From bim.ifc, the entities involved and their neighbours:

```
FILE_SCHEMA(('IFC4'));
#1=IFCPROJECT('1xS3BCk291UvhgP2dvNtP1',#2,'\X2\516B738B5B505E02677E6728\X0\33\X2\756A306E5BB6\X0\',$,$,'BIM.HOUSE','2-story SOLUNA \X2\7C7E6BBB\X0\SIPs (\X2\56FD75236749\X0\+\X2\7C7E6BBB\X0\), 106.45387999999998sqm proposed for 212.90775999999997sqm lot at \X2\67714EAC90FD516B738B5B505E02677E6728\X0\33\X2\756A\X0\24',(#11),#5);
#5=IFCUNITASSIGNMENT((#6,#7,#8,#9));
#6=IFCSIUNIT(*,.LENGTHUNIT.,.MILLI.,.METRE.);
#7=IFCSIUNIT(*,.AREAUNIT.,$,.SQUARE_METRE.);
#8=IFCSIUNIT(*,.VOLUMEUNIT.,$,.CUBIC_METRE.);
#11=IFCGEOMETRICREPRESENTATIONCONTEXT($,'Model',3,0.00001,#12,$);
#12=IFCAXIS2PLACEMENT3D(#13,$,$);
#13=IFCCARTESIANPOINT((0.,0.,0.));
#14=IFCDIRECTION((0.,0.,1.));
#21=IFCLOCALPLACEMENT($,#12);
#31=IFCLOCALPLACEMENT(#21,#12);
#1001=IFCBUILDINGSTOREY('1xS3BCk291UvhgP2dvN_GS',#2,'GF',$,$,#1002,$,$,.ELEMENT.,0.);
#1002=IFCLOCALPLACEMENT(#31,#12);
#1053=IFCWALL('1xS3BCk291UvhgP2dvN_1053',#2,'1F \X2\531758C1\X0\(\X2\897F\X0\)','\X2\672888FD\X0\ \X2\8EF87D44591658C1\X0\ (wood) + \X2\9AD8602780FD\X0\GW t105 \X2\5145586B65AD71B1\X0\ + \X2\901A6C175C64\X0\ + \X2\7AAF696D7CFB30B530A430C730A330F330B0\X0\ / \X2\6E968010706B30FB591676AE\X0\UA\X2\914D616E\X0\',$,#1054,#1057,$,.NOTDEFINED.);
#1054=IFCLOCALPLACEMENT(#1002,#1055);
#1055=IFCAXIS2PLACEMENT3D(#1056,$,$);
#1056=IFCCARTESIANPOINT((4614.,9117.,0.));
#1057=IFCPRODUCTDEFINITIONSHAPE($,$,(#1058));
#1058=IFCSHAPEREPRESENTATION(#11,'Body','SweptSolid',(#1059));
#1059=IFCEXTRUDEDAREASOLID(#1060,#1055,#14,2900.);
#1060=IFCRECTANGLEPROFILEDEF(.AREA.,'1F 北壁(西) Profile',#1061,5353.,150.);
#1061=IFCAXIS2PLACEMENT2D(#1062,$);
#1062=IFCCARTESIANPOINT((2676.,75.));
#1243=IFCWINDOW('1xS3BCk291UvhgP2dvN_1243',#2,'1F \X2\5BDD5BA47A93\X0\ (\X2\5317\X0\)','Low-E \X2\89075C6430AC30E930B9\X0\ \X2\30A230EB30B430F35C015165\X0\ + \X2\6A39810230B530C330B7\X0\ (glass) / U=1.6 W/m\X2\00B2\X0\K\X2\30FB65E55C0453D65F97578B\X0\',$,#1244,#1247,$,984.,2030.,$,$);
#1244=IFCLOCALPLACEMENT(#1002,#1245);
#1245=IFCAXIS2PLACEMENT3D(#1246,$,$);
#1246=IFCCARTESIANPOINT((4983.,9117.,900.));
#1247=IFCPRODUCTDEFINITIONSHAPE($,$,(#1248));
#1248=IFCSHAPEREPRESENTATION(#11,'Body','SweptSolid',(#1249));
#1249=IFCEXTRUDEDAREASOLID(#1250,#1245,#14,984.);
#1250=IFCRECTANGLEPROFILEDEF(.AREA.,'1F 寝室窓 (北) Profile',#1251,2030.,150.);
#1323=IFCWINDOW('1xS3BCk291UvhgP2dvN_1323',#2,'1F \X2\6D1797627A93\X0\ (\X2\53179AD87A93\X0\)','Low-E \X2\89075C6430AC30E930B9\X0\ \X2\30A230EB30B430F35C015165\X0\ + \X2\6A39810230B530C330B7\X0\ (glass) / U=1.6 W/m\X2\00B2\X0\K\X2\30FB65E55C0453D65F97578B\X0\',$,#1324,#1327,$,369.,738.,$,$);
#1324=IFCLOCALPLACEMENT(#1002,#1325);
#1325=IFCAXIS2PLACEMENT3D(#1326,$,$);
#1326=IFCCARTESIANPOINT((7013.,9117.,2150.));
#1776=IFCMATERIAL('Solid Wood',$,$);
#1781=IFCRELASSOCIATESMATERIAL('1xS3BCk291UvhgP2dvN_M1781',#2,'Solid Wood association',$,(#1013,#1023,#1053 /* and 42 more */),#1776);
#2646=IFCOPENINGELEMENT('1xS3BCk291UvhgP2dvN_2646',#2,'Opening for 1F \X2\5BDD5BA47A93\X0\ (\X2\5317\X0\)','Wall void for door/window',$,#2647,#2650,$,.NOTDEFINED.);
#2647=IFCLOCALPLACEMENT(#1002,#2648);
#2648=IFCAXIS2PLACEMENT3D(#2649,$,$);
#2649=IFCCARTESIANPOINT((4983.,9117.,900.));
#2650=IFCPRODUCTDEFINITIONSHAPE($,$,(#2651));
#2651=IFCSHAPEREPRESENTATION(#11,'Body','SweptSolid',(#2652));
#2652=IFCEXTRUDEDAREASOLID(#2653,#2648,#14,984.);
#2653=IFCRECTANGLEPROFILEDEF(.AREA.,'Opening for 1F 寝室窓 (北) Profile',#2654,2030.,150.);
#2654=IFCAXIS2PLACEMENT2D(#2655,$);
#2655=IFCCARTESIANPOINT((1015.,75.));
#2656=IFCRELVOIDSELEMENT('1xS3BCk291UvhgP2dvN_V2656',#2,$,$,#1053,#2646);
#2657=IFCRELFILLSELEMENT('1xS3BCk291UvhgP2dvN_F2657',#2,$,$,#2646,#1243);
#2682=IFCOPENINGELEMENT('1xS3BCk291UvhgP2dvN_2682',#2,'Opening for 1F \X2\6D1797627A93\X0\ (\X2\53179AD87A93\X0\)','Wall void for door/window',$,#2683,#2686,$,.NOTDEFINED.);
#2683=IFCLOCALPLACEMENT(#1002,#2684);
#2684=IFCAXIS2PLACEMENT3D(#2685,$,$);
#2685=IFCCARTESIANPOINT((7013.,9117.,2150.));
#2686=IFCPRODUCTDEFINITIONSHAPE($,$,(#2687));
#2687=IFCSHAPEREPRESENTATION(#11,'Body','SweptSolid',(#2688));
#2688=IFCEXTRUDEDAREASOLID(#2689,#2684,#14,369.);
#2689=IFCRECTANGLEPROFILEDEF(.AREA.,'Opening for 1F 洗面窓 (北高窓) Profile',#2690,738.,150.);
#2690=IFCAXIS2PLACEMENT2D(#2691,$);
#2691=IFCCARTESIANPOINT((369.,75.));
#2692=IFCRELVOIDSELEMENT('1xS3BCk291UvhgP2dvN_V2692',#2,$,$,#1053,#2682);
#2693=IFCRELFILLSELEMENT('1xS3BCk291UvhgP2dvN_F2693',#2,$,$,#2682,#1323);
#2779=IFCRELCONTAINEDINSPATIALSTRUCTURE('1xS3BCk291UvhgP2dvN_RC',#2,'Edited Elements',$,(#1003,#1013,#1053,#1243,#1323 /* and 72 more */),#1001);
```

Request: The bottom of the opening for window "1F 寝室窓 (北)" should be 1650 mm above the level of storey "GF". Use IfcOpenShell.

```python
import numpy as np
import ifcopenshell
import ifcopenshell.api.geometry
import ifcopenshell.geom
import ifcopenshell.util.element
import ifcopenshell.util.placement
import ifcopenshell.util.shape
import ifcopenshell.util.unit

model = ifcopenshell.open("bim.ifc")
unit_scale = ifcopenshell.util.unit.calculate_unit_scale(model)

window = model.by_guid("1xS3BCk291UvhgP2dvN_1243")
opening = window.FillsVoids[0].RelatingOpeningElement
storey = ifcopenshell.util.element.get_container(window, ifc_class="IfcBuildingStorey")
level = ifcopenshell.util.placement.get_local_placement(storey.ObjectPlacement)[2, 3]

# The opening's origin need not be at the sill, so measure its lowest point.
shape = ifcopenshell.geom.create_shape(ifcopenshell.geom.settings(), opening)
bottom = ifcopenshell.util.shape.get_shape_bottom_elevation(shape, shape.geometry) / unit_scale
dz = level + 1650.0 - bottom

shift = np.array([0.0, 0.0, dz])
# The window is not placed relative to its opening, so move both.
for product in (opening, window):
    matrix = ifcopenshell.util.placement.get_local_placement(product.ObjectPlacement)
    matrix[:3, 3] += shift
    ifcopenshell.api.geometry.edit_object_placement(model, product=product, matrix=matrix, is_si=False)

print(f"moved by {dz * unit_scale:+.3f} m")

model.write("bim_rev.ifc")
```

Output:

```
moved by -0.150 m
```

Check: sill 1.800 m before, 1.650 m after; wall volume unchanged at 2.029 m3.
